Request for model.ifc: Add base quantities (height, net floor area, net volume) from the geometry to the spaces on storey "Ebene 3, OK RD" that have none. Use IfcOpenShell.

First a look at what the model holds.

```python
import ifcopenshell
import ifcopenshell.util.element
import ifcopenshell.util.unit

model = ifcopenshell.open("model.ifc")
print(model.schema)
for unit_type in ("LENGTHUNIT", "AREAUNIT", "VOLUMEUNIT"):
    print(unit_type, ifcopenshell.util.unit.calculate_unit_scale(model, unit_type))
storey = next(s for s in model.by_type("IfcBuildingStorey") if s.Name == "Ebene 3, OK RD")
spaces = [e for e in ifcopenshell.util.element.get_decomposition(storey) if e.is_a("IfcSpace")]
for e in sorted(spaces, key=lambda e: e.id()):
    print(e.id(), e.is_a(), e.Name, list(ifcopenshell.util.element.get_psets(e, qtos_only=True)), sep=" | ")
```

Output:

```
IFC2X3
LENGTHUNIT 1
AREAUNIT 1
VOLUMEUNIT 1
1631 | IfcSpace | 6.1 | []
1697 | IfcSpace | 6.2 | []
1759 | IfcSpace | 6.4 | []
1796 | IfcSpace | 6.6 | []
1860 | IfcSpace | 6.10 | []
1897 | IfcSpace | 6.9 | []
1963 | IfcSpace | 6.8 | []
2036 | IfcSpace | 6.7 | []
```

```python
import ifcopenshell
import ifcopenshell.api.pset
import ifcopenshell.geom
import ifcopenshell.util.element
import ifcopenshell.util.shape
import ifcopenshell.util.unit

model = ifcopenshell.open("model.ifc")
unit_scale = ifcopenshell.util.unit.calculate_unit_scale(model)
area_scale = ifcopenshell.util.unit.calculate_unit_scale(model, "AREAUNIT")
volume_scale = ifcopenshell.util.unit.calculate_unit_scale(model, "VOLUMEUNIT")
settings = ifcopenshell.geom.settings()

storey = next(s for s in model.by_type("IfcBuildingStorey") if s.Name == "Ebene 3, OK RD")
spaces = [e for e in ifcopenshell.util.element.get_decomposition(storey) if e.is_a("IfcSpace")]

for e in sorted(spaces, key=lambda e: e.id()):
    if ifcopenshell.util.element.get_psets(e, qtos_only=True, should_inherit=False):
        continue
    # Geometry comes back in metres, in the element's own axes.
    shape = ifcopenshell.geom.create_shape(settings, e)
    values = {
        "Height": ifcopenshell.util.shape.get_z(shape.geometry) / unit_scale,
        "NetFloorArea": ifcopenshell.util.shape.get_footprint_area(shape.geometry) / area_scale,
        "NetVolume": ifcopenshell.util.shape.get_volume(shape.geometry) / volume_scale,
    }
    qto = ifcopenshell.api.pset.add_qto(model, product=e, name="BaseQuantities")
    ifcopenshell.api.pset.edit_qto(model, qto=qto, properties=values)
    print(e.id(), {k: round(v, 3) for k, v in values.items()})

model.write("model_rev.ifc")
```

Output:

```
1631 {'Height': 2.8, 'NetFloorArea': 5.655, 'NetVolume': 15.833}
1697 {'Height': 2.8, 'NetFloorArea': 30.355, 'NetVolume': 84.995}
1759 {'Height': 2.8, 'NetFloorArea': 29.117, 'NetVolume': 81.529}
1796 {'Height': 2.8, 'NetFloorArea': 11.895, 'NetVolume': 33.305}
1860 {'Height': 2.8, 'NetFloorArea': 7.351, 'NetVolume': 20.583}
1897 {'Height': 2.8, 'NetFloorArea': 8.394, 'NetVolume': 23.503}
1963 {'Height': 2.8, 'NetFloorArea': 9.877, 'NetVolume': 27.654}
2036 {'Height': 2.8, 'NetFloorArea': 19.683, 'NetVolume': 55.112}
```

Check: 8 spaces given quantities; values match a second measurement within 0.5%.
